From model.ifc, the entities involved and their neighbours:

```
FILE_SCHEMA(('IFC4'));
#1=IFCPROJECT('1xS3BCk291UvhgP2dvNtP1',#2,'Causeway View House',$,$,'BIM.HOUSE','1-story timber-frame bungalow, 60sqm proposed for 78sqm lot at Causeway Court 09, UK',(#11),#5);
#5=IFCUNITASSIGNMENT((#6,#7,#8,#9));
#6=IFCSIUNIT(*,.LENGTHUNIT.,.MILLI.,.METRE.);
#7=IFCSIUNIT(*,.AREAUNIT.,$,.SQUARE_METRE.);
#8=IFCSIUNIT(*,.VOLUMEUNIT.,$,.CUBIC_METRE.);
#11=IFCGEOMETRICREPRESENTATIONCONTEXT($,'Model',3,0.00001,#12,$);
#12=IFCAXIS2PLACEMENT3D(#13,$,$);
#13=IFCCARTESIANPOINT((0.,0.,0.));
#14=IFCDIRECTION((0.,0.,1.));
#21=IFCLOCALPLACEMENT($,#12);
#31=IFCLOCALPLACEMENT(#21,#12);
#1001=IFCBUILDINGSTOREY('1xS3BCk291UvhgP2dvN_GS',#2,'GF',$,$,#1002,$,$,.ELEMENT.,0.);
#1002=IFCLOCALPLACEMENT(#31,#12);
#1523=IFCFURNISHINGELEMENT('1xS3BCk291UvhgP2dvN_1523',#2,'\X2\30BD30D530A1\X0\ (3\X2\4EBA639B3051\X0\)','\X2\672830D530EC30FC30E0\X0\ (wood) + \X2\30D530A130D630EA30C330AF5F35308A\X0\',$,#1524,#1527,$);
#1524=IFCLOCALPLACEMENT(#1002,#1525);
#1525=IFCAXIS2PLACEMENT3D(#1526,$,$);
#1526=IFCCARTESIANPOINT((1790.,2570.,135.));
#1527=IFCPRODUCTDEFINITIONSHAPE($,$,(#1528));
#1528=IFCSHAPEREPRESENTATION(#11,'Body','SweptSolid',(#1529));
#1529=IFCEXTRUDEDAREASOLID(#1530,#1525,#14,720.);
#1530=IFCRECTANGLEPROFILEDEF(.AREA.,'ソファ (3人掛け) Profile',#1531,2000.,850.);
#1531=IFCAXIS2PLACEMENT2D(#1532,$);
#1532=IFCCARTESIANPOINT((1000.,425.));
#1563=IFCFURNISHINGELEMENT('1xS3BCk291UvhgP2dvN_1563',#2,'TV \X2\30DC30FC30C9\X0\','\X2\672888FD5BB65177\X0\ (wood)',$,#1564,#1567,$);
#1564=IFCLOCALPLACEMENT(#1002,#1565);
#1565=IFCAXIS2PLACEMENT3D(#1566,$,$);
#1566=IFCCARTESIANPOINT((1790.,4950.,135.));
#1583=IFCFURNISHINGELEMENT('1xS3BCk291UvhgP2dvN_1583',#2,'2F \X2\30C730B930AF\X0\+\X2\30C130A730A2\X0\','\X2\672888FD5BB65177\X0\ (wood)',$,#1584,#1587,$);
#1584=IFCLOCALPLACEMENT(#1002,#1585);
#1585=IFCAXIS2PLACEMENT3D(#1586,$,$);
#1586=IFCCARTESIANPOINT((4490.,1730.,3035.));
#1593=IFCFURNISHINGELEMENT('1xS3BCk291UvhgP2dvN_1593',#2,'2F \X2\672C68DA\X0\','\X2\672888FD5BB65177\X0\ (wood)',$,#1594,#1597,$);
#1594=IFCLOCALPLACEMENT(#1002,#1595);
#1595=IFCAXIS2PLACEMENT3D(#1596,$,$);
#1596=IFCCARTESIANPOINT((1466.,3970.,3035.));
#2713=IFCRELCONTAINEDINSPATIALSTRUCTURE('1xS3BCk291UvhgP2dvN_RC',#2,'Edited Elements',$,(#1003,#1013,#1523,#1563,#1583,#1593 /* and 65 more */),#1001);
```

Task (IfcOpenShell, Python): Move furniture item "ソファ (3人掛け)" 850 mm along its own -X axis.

```python
import ifcopenshell
import ifcopenshell.api.geometry
import ifcopenshell.util.placement

model = ifcopenshell.open("model.ifc")

item = model.by_id(1523)
matrix = ifcopenshell.util.placement.get_local_placement(item.ObjectPlacement)
matrix[:3, 3] -= matrix[:3, 0] * 850.0
ifcopenshell.api.geometry.edit_object_placement(model, product=item, matrix=matrix, is_si=False)

print(ifcopenshell.util.placement.get_local_placement(item.ObjectPlacement).round(3) + 0.0)

model.write("model_edited.ifc")
```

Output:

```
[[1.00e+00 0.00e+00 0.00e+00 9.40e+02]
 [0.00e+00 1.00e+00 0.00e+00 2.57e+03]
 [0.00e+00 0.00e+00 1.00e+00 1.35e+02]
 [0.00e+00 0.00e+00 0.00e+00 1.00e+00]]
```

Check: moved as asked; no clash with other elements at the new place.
